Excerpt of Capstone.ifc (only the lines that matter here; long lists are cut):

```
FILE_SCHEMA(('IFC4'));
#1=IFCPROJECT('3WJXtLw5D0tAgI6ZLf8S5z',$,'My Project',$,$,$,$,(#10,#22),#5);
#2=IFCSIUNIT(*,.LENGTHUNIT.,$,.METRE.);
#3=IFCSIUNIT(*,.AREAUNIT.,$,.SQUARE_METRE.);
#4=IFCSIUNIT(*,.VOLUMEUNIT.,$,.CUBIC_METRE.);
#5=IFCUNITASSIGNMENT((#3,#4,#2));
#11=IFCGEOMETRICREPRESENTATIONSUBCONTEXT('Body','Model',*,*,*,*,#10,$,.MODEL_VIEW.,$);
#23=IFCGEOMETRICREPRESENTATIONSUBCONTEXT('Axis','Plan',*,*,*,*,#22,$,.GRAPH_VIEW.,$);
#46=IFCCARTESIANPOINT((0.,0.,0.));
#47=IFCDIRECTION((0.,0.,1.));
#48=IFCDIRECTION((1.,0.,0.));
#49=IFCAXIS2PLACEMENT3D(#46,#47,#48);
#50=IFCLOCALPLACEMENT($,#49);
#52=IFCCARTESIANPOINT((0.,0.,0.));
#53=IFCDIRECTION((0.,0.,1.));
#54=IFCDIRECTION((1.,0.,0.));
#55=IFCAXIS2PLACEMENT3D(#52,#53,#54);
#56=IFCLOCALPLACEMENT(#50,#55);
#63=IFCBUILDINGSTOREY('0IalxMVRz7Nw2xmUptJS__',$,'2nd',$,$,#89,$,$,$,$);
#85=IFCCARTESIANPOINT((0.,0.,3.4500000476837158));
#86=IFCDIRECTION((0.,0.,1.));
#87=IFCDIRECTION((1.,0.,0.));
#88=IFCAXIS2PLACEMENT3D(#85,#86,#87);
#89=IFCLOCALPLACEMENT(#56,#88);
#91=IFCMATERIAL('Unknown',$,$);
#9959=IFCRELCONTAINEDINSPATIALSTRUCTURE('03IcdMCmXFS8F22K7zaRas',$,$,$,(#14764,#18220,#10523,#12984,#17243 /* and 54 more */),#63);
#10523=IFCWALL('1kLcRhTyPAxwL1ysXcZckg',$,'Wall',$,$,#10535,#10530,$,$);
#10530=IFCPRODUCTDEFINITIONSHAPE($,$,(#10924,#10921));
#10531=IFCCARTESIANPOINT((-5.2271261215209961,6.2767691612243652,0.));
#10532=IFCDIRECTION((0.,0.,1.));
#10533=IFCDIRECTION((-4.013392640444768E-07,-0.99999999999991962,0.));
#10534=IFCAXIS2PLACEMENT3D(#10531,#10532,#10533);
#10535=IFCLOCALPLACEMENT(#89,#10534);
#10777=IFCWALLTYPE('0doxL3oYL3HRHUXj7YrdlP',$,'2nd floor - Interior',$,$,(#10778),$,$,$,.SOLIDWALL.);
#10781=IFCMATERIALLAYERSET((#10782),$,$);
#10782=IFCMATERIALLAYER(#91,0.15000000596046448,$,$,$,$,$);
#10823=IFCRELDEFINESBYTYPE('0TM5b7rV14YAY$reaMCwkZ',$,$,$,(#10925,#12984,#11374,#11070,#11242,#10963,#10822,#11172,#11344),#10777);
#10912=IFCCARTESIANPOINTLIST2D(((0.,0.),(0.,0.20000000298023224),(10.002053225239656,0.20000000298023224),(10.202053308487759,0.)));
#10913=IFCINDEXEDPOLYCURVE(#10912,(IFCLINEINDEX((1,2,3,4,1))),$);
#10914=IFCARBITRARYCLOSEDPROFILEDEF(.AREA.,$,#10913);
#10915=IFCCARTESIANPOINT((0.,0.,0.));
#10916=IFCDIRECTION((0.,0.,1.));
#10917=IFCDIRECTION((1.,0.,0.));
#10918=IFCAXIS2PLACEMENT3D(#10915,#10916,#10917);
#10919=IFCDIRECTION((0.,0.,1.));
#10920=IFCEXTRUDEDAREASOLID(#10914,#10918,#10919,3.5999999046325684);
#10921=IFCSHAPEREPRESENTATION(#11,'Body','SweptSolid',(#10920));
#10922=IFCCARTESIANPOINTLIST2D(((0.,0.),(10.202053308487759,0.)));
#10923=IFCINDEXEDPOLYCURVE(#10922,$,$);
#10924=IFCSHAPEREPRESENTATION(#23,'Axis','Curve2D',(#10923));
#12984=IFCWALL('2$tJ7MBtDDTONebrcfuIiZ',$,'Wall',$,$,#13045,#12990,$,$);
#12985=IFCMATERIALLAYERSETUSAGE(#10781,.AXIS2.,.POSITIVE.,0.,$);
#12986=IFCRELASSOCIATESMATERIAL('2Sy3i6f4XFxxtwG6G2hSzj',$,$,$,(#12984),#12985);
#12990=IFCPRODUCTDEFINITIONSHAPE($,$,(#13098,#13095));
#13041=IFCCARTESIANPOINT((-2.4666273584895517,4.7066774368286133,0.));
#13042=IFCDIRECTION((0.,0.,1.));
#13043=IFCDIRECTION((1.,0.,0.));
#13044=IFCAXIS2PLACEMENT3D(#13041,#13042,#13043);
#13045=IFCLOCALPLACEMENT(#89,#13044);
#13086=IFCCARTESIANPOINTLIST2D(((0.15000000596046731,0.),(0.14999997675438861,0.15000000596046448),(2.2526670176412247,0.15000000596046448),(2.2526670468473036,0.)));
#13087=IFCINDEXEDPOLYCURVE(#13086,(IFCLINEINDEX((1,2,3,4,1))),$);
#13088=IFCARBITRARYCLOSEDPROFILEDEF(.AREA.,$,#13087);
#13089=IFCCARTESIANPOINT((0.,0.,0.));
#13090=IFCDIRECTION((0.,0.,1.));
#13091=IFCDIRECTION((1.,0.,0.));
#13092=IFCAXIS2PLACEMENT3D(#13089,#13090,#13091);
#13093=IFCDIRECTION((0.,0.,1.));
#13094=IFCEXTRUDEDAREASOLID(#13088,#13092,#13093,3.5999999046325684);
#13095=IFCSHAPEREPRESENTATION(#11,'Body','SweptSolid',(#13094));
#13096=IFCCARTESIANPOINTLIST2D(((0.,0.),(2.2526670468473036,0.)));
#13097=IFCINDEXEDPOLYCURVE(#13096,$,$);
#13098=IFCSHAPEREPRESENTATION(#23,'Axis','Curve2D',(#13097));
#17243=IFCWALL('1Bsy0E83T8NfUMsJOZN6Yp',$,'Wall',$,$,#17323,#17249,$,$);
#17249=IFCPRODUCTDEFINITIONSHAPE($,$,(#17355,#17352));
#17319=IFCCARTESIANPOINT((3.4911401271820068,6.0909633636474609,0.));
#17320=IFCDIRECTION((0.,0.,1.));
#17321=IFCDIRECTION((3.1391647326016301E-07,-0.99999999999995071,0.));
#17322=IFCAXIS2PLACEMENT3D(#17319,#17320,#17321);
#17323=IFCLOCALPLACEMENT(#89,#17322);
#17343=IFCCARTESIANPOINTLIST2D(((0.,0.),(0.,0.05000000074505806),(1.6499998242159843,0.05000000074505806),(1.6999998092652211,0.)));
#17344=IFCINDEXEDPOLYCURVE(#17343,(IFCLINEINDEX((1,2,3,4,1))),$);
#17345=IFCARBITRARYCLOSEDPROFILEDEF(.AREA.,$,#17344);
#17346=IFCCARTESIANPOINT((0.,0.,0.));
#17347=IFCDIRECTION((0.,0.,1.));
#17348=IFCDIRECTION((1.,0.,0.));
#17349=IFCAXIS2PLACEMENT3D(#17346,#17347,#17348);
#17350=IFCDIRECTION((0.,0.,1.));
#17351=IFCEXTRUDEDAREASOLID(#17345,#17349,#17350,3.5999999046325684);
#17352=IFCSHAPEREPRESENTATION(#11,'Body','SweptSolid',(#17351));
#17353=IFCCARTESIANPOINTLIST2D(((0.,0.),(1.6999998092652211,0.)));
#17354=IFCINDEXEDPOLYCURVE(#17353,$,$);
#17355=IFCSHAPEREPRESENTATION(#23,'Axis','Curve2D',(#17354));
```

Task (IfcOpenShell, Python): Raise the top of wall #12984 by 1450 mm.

```python
import ifcopenshell
import ifcopenshell.geom
import ifcopenshell.util.representation
import ifcopenshell.util.shape

model = ifcopenshell.open("Capstone.ifc")
settings = ifcopenshell.geom.settings()


def volume(element):
    """Net volume in cubic metres, openings subtracted."""
    shape = ifcopenshell.geom.create_shape(settings, element)
    return ifcopenshell.util.shape.get_volume(shape.geometry)


wall = model.by_guid("2$tJ7MBtDDTONebrcfuIiZ")
before = volume(wall)

body = ifcopenshell.util.representation.get_representation(wall, "Model", "Body")
solid = body.Items[0]
old_height = solid.Depth
solid.Depth += 1.45
after = volume(wall)

print(f"height {old_height:g} -> {solid.Depth:g}, volume {before:.3f} -> {after:.3f} m3")

model.write("Capstone_rev.ifc")
```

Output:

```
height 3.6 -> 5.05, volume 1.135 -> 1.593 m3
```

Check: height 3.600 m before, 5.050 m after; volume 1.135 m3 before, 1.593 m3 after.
